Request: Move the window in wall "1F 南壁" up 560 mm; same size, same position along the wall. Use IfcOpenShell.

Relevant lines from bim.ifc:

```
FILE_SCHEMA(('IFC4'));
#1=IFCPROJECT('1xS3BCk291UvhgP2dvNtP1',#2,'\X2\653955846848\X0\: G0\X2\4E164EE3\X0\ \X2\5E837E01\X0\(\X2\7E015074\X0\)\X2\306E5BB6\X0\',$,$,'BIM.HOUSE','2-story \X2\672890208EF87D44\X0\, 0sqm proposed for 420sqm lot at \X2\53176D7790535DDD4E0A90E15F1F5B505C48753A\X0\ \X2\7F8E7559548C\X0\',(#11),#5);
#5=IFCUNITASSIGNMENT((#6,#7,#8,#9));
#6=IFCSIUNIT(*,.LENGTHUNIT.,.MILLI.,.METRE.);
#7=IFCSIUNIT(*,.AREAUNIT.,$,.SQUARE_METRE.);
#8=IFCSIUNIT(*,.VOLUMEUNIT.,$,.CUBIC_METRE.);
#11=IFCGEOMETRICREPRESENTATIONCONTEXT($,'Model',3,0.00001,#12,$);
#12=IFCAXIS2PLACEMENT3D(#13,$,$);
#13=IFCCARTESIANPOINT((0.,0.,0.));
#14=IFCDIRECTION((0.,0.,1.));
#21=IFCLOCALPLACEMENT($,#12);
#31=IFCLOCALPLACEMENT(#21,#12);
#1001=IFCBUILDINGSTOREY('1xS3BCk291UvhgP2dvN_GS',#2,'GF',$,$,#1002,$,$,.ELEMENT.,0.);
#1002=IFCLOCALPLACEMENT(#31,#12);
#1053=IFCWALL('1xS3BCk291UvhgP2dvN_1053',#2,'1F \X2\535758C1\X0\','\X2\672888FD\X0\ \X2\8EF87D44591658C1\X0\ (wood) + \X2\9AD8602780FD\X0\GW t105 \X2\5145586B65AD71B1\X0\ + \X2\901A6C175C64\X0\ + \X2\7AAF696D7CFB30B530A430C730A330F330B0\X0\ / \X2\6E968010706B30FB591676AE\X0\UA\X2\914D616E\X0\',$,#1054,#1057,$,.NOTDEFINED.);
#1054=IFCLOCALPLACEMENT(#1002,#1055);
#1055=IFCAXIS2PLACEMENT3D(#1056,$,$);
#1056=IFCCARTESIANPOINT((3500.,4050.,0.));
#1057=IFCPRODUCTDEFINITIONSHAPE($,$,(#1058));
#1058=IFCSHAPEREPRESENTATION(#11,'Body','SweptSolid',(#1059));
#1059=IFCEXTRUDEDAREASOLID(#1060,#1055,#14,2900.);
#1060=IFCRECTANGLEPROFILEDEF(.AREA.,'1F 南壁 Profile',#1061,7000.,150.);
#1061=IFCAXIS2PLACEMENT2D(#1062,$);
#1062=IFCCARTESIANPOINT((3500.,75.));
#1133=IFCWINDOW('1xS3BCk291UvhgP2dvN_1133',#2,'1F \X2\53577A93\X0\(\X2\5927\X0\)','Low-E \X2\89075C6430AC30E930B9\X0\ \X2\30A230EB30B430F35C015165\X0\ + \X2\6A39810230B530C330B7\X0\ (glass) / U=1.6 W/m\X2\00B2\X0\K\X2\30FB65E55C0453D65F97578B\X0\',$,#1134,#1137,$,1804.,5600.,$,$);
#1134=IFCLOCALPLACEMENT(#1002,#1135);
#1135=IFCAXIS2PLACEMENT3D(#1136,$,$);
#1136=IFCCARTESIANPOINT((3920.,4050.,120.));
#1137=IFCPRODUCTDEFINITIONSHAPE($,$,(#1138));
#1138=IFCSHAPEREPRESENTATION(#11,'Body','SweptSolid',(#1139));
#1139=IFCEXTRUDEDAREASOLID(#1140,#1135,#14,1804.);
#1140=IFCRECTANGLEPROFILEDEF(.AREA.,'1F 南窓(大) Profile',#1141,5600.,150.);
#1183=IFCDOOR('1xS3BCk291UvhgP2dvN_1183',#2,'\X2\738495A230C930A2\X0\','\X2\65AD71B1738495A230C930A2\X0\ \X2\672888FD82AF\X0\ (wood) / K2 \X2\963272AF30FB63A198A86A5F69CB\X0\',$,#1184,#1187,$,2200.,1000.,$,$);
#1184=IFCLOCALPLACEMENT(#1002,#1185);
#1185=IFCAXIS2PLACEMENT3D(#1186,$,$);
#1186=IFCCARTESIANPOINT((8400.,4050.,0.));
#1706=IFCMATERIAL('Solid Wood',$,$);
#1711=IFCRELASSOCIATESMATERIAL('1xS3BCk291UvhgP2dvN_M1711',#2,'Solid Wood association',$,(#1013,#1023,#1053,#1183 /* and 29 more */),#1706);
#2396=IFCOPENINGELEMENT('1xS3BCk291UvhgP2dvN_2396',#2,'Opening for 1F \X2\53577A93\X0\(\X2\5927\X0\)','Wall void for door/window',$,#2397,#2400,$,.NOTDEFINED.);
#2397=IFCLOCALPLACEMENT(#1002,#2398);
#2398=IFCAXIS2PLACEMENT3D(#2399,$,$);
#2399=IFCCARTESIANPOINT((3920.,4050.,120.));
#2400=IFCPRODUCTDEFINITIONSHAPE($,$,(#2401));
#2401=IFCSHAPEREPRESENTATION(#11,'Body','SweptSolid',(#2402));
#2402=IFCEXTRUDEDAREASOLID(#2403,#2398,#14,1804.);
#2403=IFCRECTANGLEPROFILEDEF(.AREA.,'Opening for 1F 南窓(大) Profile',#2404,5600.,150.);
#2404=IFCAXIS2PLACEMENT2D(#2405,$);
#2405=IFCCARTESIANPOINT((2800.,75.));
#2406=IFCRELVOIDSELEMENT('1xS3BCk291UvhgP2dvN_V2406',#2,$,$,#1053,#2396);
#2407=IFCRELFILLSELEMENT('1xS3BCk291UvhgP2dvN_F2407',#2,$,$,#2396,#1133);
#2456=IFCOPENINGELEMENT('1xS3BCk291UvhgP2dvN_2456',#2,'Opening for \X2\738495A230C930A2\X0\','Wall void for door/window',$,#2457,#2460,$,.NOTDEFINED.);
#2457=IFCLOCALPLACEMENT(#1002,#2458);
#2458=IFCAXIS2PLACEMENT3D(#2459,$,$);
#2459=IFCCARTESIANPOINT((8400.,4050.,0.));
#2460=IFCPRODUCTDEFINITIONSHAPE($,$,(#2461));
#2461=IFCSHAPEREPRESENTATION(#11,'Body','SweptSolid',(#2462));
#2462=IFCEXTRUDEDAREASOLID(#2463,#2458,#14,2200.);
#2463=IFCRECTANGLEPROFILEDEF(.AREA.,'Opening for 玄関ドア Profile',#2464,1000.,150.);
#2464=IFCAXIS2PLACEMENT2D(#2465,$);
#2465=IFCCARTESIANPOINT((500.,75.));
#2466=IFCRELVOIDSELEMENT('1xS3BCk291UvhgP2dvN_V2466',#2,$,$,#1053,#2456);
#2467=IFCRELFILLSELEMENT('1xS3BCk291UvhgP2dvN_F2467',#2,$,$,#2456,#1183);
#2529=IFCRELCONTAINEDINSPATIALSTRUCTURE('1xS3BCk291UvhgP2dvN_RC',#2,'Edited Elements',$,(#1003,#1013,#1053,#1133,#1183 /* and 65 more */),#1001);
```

```python
import numpy as np
import ifcopenshell
import ifcopenshell.api.geometry
import ifcopenshell.util.placement
import ifcopenshell.util.unit

model = ifcopenshell.open("bim.ifc")
unit_scale = ifcopenshell.util.unit.calculate_unit_scale(model)

window = model.by_guid("1xS3BCk291UvhgP2dvN_1133")
opening = window.FillsVoids[0].RelatingOpeningElement
dz = 0.56 / unit_scale

shift = np.array([0.0, 0.0, dz])
# The window is not placed relative to its opening, so move both.
for product in (opening, window):
    matrix = ifcopenshell.util.placement.get_local_placement(product.ObjectPlacement)
    matrix[:3, 3] += shift
    ifcopenshell.api.geometry.edit_object_placement(model, product=product, matrix=matrix, is_si=False)

print(f"moved by {dz * unit_scale:+.3f} m")

model.write("bim_rev.ifc")
```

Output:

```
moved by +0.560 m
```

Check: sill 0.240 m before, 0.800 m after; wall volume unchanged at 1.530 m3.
